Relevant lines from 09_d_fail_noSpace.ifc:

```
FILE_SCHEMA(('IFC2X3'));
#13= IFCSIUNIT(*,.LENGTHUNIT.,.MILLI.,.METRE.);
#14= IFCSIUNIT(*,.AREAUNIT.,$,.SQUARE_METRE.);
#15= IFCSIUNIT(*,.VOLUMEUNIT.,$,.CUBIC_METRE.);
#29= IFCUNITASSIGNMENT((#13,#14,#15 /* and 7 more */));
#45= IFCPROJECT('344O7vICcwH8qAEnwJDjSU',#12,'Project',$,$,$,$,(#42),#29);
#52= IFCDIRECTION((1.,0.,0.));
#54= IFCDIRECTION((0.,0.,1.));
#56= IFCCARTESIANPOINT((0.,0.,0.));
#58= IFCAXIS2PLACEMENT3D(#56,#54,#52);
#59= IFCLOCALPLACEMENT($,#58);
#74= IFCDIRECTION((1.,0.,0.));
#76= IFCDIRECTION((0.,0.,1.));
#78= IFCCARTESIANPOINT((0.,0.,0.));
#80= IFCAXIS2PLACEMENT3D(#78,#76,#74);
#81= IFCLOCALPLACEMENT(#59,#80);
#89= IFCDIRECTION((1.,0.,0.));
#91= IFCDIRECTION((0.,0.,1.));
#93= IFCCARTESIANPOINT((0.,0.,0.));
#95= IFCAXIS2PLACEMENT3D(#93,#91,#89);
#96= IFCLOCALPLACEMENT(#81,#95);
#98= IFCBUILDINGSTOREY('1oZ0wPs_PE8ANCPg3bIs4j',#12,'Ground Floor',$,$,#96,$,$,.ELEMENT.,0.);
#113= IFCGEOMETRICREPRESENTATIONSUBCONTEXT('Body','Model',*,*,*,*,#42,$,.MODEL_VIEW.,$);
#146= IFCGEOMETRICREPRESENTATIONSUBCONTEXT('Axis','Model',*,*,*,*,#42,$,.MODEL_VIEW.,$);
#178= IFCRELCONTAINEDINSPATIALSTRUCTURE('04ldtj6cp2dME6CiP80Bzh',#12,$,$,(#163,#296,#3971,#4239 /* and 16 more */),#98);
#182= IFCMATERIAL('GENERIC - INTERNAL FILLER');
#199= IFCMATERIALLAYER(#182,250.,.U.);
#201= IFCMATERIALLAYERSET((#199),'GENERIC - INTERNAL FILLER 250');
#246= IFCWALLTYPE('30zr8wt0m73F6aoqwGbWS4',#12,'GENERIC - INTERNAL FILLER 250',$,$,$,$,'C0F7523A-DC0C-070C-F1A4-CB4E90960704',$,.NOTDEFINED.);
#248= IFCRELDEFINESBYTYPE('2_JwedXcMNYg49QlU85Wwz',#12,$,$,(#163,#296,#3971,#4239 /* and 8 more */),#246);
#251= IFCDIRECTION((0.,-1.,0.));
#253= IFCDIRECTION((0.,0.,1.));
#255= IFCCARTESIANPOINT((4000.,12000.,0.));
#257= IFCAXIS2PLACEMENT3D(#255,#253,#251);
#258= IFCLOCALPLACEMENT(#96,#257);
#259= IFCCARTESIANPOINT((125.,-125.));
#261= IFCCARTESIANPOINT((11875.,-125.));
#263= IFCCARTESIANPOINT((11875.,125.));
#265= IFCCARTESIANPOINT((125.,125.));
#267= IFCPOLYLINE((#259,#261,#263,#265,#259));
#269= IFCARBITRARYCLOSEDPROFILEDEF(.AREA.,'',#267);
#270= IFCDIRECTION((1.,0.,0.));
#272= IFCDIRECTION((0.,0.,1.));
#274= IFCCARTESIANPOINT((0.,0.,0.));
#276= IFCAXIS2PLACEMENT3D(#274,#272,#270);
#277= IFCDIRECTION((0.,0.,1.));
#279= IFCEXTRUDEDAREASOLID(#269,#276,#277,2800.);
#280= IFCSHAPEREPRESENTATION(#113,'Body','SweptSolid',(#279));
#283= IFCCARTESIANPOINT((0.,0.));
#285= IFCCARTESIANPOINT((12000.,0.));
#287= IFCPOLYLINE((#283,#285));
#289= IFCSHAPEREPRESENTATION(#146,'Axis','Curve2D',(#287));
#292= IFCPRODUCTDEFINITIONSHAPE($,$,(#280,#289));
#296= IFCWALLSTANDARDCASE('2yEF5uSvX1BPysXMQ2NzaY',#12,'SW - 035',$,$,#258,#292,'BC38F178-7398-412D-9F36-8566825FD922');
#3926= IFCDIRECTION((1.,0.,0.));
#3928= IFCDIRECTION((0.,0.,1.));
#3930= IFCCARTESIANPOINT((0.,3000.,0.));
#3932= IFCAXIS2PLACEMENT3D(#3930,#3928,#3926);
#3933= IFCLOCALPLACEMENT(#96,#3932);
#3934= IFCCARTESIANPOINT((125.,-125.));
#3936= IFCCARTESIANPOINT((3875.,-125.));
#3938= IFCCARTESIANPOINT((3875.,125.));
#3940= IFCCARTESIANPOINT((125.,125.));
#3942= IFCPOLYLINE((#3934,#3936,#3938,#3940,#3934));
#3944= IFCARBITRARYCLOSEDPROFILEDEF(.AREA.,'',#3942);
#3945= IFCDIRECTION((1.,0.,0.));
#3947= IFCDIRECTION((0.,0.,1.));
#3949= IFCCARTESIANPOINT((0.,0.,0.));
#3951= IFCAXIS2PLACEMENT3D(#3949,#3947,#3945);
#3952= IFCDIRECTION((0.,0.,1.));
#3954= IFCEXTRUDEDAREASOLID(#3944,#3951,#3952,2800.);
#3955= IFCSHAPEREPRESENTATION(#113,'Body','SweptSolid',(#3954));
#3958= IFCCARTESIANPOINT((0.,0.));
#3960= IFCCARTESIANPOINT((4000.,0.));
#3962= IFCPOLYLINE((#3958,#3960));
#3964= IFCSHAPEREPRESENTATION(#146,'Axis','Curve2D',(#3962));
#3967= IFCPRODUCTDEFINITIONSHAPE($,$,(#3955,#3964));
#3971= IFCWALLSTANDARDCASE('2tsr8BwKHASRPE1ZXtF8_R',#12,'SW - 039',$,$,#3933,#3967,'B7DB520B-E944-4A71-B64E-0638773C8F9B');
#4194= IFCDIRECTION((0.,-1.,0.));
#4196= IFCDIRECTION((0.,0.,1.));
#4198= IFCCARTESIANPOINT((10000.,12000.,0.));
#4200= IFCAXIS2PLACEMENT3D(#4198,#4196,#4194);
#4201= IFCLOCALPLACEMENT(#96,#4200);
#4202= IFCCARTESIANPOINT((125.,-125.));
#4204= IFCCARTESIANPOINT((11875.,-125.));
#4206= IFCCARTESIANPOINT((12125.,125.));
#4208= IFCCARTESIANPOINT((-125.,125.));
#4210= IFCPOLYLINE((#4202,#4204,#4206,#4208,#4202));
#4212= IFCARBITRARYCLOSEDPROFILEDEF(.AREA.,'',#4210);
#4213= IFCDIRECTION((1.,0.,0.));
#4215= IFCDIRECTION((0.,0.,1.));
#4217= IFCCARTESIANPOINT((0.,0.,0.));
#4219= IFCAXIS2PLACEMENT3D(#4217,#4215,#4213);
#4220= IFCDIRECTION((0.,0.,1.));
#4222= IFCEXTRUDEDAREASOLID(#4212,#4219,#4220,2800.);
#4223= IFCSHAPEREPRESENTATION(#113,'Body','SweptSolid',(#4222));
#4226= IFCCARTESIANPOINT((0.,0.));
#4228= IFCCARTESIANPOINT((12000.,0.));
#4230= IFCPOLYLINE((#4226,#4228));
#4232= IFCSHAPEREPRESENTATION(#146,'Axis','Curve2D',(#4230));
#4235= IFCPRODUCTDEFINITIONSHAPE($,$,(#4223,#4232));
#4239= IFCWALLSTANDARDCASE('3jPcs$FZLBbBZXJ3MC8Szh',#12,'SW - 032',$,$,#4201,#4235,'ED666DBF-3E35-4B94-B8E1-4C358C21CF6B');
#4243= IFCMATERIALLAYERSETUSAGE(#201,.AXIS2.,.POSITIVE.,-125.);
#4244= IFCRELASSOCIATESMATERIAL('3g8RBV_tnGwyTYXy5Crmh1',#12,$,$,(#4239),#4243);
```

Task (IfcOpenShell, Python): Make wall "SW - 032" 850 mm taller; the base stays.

```python
import ifcopenshell
import ifcopenshell.geom
import ifcopenshell.util.representation
import ifcopenshell.util.shape
import ifcopenshell.util.unit

model = ifcopenshell.open("09_d_fail_noSpace.ifc")
unit_scale = ifcopenshell.util.unit.calculate_unit_scale(model)
settings = ifcopenshell.geom.settings()


def volume(element):
    """Net volume in cubic metres, openings subtracted."""
    shape = ifcopenshell.geom.create_shape(settings, element)
    return ifcopenshell.util.shape.get_volume(shape.geometry)


wall = model.by_guid("3jPcs$FZLBbBZXJ3MC8Szh")
before = volume(wall)

body = ifcopenshell.util.representation.get_representation(wall, "Model", "Body")
solid = body.Items[0]
old_height = solid.Depth
solid.Depth += 0.85 / unit_scale
after = volume(wall)

print(f"height {old_height:g} -> {solid.Depth:g}, volume {before:.3f} -> {after:.3f} m3")

model.write("09_d_fail_noSpace_edited.ifc")
```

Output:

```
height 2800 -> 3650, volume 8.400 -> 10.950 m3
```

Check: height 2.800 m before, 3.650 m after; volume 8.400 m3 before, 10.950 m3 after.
